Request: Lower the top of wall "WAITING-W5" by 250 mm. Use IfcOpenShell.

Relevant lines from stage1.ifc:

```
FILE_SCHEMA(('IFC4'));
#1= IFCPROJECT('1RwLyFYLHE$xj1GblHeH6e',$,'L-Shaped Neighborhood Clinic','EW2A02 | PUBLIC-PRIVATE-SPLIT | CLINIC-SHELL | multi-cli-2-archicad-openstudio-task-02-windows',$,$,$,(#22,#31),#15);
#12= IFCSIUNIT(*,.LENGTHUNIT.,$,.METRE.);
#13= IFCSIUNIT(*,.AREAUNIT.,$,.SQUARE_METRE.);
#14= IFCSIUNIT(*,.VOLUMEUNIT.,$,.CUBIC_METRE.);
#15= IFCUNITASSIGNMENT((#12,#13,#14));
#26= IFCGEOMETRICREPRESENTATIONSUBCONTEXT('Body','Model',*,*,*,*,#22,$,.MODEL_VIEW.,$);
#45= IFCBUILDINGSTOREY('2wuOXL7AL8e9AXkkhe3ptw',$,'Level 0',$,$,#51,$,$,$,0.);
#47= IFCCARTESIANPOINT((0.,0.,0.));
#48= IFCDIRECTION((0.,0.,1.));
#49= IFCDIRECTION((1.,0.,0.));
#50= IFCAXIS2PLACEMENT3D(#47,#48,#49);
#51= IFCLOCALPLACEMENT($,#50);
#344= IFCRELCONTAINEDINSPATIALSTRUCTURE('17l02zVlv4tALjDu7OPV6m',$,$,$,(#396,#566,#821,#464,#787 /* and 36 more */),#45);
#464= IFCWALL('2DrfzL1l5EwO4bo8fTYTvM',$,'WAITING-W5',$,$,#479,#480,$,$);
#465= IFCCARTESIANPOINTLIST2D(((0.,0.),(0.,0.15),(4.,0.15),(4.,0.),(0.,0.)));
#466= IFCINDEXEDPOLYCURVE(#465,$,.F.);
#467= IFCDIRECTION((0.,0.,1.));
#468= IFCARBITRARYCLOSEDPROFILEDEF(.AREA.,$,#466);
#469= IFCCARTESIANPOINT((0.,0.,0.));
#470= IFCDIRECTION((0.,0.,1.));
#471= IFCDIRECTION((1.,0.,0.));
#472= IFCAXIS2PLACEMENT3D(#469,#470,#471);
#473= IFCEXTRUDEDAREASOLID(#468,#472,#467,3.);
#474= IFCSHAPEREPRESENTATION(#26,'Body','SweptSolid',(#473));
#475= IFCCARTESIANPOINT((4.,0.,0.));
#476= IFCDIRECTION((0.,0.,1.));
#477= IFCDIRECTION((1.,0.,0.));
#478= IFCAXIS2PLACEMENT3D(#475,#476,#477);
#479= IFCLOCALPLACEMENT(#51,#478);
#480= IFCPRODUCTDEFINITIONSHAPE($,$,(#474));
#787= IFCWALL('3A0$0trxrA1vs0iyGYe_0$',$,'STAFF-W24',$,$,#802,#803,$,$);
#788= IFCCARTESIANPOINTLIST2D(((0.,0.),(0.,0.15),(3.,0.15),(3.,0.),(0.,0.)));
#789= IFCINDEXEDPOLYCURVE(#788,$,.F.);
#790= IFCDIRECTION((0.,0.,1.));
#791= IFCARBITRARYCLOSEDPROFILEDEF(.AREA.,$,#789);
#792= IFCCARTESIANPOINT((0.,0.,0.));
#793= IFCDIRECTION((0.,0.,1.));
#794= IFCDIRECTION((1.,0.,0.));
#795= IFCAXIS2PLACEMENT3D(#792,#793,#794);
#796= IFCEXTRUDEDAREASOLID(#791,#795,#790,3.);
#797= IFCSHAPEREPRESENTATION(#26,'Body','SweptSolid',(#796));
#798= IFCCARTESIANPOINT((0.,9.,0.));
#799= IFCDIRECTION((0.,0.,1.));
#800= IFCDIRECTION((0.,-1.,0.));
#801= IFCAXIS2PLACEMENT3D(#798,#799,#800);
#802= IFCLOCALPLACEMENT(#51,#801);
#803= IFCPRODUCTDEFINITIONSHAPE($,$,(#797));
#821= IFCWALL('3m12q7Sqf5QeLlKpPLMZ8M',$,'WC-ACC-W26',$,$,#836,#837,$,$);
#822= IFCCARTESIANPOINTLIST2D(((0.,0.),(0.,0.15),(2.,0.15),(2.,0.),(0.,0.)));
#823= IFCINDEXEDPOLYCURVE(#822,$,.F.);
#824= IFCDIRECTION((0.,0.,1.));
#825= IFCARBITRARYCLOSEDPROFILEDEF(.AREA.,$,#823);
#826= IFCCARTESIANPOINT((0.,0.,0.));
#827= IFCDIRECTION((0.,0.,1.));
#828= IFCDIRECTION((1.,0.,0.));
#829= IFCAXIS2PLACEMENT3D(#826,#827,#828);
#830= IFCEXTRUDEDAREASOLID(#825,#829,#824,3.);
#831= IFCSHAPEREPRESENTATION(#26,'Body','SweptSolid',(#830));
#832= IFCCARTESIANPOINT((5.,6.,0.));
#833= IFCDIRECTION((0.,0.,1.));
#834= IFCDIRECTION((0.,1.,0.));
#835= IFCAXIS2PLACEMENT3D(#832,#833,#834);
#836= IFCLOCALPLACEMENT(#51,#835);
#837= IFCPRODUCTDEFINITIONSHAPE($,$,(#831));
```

```python
import ifcopenshell
import ifcopenshell.geom
import ifcopenshell.util.representation
import ifcopenshell.util.shape
import ifcopenshell.util.unit

model = ifcopenshell.open("stage1.ifc")
unit_scale = ifcopenshell.util.unit.calculate_unit_scale(model)
settings = ifcopenshell.geom.settings()


def volume(element):
    """Net volume in cubic metres, openings subtracted."""
    shape = ifcopenshell.geom.create_shape(settings, element)
    return ifcopenshell.util.shape.get_volume(shape.geometry)


wall = model.by_guid("2DrfzL1l5EwO4bo8fTYTvM")
before = volume(wall)

body = ifcopenshell.util.representation.get_representation(wall, "Model", "Body")
solid = body.Items[0]
old_height = solid.Depth
solid.Depth -= 0.25 / unit_scale
after = volume(wall)

print(f"height {old_height:g} -> {solid.Depth:g}, volume {before:.3f} -> {after:.3f} m3")

model.write("stage1_rev.ifc")
```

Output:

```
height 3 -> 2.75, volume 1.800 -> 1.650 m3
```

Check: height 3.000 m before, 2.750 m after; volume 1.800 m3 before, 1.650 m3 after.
